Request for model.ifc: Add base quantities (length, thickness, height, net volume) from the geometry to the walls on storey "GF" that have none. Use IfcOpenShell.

First a look at what the model holds.

```python
import ifcopenshell
import ifcopenshell.util.element
import ifcopenshell.util.unit

model = ifcopenshell.open("model.ifc")
print(model.schema)
for unit_type in ("LENGTHUNIT", "AREAUNIT", "VOLUMEUNIT"):
    print(unit_type, ifcopenshell.util.unit.calculate_unit_scale(model, unit_type))
storey = next(s for s in model.by_type("IfcBuildingStorey") if s.Name == "GF")
walls = [e for e in ifcopenshell.util.element.get_decomposition(storey) if e.is_a("IfcWall")]
for e in sorted(walls, key=lambda e: e.id()):
    print(e.id(), e.is_a(), e.Name, list(ifcopenshell.util.element.get_psets(e, qtos_only=True)), sep=" | ")
```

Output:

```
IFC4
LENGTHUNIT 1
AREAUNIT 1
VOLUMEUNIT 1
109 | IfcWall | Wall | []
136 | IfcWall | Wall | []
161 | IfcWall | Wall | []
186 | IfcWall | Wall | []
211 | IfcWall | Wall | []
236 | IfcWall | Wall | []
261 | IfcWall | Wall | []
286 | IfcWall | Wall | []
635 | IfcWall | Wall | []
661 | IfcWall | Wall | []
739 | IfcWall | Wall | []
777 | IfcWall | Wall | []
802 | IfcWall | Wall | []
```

```python
import ifcopenshell
import ifcopenshell.api.pset
import ifcopenshell.geom
import ifcopenshell.util.element
import ifcopenshell.util.shape
import ifcopenshell.util.unit

model = ifcopenshell.open("model.ifc")
unit_scale = ifcopenshell.util.unit.calculate_unit_scale(model)
volume_scale = ifcopenshell.util.unit.calculate_unit_scale(model, "VOLUMEUNIT")
settings = ifcopenshell.geom.settings()

storey = next(s for s in model.by_type("IfcBuildingStorey") if s.Name == "GF")
walls = [e for e in ifcopenshell.util.element.get_decomposition(storey) if e.is_a("IfcWall")]

for e in sorted(walls, key=lambda e: e.id()):
    if ifcopenshell.util.element.get_psets(e, qtos_only=True, should_inherit=False):
        continue
    # Geometry comes back in metres, in the element's own axes.
    shape = ifcopenshell.geom.create_shape(settings, e)
    values = {
        "Length": ifcopenshell.util.shape.get_x(shape.geometry) / unit_scale,
        "Width": ifcopenshell.util.shape.get_y(shape.geometry) / unit_scale,
        "Height": ifcopenshell.util.shape.get_z(shape.geometry) / unit_scale,
        "NetVolume": ifcopenshell.util.shape.get_volume(shape.geometry) / volume_scale,
    }
    qto = ifcopenshell.api.pset.add_qto(model, product=e, name="Qto_WallBaseQuantities")
    ifcopenshell.api.pset.edit_qto(model, qto=qto, properties=values)
    print(e.id(), {k: round(v, 3) for k, v in values.items()})

model.write("model_v2.ifc")
```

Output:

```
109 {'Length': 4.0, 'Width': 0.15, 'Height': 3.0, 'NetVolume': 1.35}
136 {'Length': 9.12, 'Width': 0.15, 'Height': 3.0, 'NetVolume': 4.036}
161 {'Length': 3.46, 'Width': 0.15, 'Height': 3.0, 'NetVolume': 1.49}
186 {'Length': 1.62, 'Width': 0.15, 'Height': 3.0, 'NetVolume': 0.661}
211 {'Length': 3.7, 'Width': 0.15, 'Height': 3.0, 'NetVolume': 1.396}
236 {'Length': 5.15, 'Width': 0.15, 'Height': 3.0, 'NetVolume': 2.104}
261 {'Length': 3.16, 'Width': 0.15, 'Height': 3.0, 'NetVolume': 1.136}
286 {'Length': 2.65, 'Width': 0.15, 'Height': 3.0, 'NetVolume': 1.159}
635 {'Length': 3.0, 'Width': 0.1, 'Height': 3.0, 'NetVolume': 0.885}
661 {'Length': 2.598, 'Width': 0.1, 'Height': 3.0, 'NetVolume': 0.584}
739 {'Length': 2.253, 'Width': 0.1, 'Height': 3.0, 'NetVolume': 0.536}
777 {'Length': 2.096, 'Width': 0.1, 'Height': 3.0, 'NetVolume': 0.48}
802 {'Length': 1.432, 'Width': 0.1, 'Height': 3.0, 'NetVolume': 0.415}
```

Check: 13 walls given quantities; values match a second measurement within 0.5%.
